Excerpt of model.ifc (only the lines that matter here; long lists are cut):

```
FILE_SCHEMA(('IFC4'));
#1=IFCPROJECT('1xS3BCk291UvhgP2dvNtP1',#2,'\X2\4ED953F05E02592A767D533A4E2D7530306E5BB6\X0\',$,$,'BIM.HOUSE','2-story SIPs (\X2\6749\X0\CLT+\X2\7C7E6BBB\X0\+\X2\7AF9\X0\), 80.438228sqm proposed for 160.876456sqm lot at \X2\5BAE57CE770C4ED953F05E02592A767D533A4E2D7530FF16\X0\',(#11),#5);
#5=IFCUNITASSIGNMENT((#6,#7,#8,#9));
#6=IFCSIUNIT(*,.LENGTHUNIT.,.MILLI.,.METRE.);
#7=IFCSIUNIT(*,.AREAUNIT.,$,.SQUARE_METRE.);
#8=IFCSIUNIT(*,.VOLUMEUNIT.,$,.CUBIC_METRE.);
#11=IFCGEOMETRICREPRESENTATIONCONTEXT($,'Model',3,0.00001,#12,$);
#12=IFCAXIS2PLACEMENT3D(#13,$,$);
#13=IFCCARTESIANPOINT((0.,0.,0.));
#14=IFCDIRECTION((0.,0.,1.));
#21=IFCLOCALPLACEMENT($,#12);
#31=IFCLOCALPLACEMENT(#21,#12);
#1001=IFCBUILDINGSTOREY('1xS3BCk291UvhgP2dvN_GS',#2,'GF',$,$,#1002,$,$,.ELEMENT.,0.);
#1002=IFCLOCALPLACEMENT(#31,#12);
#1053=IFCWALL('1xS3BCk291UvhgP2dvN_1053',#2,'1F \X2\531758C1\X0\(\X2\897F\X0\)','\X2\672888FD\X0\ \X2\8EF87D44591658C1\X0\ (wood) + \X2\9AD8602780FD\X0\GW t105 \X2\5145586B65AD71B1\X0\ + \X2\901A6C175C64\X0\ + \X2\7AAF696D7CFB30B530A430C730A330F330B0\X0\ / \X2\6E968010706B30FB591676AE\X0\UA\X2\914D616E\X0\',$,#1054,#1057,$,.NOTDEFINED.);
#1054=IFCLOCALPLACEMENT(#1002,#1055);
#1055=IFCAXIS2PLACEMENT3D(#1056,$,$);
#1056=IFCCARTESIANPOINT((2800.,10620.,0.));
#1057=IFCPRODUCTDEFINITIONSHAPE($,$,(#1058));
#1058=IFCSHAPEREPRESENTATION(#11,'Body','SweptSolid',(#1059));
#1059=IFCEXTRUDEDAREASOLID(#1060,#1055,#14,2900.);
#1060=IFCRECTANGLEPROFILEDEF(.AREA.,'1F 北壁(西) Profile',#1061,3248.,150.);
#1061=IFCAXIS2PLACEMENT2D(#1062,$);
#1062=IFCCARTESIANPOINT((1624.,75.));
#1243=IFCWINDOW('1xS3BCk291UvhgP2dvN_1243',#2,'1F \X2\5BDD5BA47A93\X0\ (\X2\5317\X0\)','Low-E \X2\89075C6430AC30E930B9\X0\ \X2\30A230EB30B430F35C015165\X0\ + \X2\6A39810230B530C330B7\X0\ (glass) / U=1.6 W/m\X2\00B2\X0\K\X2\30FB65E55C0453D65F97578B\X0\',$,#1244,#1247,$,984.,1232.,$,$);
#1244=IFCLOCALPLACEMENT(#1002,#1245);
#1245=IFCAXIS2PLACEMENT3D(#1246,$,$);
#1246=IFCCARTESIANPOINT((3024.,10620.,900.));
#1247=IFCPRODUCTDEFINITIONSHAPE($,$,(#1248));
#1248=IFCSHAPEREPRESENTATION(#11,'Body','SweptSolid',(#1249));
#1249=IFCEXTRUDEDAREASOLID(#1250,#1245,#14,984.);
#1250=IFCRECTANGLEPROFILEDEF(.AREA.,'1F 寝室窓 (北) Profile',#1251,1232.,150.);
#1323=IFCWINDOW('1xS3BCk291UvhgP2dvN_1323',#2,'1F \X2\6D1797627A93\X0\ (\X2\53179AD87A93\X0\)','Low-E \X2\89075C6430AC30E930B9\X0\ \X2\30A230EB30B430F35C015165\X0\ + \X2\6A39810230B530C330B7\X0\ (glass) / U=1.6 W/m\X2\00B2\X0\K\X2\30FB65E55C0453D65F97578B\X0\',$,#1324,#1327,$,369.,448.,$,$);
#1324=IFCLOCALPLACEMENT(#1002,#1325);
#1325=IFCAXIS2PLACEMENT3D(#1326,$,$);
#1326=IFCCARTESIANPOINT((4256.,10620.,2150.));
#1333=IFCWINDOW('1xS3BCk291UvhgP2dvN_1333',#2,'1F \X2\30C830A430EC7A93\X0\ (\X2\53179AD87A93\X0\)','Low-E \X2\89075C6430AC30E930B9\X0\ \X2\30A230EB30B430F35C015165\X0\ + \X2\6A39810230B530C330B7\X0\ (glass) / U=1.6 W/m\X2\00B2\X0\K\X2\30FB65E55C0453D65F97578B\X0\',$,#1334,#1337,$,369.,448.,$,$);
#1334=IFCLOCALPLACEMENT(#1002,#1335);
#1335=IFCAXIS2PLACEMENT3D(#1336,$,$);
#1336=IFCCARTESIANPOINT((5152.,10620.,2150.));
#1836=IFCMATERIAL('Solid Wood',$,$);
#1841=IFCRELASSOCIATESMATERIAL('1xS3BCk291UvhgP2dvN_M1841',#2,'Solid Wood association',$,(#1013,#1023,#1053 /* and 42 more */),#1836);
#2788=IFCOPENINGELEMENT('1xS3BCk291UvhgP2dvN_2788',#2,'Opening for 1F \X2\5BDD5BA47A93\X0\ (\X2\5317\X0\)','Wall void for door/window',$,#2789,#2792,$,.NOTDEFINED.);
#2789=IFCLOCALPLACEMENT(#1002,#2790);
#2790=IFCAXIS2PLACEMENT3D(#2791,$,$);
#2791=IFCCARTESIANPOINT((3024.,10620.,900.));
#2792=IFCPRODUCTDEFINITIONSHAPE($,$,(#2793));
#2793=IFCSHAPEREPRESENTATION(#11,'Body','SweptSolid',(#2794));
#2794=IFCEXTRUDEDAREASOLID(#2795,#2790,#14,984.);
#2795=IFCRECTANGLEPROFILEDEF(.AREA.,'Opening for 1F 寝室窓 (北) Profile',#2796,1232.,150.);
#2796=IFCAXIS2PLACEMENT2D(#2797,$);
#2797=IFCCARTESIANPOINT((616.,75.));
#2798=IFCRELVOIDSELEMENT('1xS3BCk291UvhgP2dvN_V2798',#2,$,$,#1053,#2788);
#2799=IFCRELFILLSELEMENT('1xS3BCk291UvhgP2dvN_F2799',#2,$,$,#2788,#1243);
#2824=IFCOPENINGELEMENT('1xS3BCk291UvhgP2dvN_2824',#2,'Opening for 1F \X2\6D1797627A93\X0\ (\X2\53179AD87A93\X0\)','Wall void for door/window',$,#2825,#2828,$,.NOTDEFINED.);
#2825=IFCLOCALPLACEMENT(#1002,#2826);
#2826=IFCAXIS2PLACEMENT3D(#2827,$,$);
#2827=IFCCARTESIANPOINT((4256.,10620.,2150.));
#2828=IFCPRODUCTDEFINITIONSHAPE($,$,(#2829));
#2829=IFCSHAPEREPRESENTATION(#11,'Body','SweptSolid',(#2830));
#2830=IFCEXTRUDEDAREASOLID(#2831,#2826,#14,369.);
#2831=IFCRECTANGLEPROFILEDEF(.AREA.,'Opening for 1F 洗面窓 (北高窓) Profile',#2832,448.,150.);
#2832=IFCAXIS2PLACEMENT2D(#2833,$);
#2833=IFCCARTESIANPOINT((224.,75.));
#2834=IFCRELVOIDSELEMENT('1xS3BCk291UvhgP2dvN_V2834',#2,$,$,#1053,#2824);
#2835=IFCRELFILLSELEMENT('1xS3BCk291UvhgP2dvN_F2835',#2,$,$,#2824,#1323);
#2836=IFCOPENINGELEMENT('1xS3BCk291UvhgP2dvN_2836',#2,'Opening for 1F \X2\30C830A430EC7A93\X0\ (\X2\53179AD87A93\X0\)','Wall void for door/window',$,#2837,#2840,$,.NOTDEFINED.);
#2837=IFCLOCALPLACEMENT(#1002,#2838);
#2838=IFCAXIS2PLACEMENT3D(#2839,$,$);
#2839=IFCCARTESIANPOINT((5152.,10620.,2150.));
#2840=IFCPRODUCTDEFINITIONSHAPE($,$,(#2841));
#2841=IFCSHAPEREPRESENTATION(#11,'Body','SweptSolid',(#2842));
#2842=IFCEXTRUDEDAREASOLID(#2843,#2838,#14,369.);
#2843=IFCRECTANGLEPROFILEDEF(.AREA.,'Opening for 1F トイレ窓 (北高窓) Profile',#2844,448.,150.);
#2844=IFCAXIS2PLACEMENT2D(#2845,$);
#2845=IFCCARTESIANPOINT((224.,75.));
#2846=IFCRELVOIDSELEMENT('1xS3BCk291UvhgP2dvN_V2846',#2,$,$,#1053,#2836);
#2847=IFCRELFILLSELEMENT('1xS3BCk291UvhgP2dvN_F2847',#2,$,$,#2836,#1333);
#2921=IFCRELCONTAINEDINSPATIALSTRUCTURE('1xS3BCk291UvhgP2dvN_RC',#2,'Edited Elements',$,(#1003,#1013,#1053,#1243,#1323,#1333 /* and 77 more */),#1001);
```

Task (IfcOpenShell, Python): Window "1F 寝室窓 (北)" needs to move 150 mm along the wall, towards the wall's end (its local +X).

```python
import ifcopenshell
import ifcopenshell.api.geometry
import ifcopenshell.util.placement
import ifcopenshell.util.unit

model = ifcopenshell.open("model.ifc")
unit_scale = ifcopenshell.util.unit.calculate_unit_scale(model)

window = model.by_guid("1xS3BCk291UvhgP2dvN_1243")
opening = window.FillsVoids[0].RelatingOpeningElement
wall = opening.VoidsElements[0].RelatingBuildingElement

wall_matrix = ifcopenshell.util.placement.get_local_placement(wall.ObjectPlacement)
shift = wall_matrix[:3, 0] * 0.15 / unit_scale
before = ifcopenshell.util.placement.get_local_placement(window.ObjectPlacement)[:3, 3].copy()

# The window is not placed relative to its opening, so move both.
for product in (opening, window):
    matrix = ifcopenshell.util.placement.get_local_placement(product.ObjectPlacement)
    matrix[:3, 3] += shift
    ifcopenshell.api.geometry.edit_object_placement(model, product=product, matrix=matrix, is_si=False)

after = ifcopenshell.util.placement.get_local_placement(window.ObjectPlacement)[:3, 3]
print("window moved by", (after - before).round(3) + 0.0)

model.write("model_updated.ifc")
```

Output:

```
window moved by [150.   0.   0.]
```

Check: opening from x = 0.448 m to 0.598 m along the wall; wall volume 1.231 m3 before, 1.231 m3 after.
